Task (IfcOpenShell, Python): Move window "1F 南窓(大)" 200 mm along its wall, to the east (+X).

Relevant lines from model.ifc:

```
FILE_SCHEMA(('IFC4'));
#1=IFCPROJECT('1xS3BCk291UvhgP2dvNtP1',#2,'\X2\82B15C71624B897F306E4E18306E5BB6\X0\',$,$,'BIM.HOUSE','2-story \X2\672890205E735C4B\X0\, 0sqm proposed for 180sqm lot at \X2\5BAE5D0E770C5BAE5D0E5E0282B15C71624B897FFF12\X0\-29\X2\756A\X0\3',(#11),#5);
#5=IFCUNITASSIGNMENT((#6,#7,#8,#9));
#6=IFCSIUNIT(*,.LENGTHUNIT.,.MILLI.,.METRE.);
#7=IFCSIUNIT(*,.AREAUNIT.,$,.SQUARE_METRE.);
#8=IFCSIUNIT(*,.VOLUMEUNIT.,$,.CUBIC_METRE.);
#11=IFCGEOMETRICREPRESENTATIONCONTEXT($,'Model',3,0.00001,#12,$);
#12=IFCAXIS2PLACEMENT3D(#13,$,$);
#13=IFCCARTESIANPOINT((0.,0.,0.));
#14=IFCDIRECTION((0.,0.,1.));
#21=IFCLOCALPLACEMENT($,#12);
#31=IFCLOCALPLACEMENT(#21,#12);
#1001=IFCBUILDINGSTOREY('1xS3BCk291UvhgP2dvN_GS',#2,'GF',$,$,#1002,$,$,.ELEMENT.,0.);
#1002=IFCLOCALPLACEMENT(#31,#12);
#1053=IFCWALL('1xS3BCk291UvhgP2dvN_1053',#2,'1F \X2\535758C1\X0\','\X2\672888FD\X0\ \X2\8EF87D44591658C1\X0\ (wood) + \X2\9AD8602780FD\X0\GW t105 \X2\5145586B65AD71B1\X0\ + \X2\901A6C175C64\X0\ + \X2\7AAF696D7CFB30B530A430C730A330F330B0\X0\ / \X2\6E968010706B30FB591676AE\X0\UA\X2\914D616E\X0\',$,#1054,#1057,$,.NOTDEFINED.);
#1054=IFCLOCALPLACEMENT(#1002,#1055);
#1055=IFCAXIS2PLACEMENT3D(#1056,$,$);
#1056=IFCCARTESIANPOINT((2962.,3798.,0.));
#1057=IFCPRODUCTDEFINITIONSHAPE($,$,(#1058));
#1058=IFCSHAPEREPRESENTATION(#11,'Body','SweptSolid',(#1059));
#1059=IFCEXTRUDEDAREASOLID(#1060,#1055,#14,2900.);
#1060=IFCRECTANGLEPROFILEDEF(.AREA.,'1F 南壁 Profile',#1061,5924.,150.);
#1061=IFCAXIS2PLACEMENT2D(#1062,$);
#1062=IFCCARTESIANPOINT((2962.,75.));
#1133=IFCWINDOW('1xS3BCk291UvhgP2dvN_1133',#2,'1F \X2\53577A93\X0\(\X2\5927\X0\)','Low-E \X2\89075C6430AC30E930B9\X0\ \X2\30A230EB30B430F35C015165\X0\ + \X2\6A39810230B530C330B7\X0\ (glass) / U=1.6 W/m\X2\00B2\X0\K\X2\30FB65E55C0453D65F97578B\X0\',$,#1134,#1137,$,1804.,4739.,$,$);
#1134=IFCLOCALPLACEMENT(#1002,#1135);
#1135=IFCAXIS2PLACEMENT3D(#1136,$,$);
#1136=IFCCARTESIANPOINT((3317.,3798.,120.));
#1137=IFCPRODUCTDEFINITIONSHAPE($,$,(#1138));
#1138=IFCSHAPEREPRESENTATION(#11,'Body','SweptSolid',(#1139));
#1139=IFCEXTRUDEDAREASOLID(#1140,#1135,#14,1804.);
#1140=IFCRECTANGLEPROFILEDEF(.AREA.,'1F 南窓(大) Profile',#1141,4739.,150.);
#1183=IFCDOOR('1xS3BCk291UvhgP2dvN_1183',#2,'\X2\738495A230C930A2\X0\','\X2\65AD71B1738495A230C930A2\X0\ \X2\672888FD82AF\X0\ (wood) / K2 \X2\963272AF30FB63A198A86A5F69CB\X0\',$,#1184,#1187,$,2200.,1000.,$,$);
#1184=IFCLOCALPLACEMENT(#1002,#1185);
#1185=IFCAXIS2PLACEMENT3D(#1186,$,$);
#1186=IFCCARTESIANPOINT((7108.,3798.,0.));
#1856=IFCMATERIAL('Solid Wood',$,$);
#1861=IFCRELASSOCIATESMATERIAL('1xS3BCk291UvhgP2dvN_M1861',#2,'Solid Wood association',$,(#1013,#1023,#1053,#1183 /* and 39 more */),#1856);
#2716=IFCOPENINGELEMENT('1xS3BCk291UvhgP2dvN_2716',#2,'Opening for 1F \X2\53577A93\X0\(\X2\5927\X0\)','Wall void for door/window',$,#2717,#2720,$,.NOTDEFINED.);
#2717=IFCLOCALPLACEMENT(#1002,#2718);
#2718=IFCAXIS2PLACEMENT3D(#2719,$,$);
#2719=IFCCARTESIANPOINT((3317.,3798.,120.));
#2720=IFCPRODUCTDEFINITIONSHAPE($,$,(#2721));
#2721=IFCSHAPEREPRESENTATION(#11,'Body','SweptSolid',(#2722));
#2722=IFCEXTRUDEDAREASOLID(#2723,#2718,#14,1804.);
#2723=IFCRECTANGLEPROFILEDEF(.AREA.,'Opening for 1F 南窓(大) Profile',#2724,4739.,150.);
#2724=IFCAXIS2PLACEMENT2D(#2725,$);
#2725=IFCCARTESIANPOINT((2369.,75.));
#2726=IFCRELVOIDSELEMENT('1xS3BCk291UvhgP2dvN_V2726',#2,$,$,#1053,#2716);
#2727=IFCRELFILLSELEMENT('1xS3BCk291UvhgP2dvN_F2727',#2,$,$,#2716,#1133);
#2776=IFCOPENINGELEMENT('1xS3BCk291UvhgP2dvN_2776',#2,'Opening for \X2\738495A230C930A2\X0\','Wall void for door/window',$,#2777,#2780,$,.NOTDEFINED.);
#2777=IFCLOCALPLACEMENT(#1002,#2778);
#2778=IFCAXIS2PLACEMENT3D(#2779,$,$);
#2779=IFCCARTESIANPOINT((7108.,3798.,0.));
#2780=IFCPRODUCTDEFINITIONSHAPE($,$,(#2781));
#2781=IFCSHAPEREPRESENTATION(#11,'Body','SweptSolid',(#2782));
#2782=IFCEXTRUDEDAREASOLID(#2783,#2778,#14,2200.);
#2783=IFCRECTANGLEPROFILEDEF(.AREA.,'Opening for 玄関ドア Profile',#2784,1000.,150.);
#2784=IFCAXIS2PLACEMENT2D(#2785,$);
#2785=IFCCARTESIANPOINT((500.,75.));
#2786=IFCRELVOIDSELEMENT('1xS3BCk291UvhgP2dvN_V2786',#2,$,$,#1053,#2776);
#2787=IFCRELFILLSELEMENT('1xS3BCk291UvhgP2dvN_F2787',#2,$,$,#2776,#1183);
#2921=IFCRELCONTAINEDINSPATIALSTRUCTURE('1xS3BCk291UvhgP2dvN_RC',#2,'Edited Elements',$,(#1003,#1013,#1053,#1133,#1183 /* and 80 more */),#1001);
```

```python
import ifcopenshell
import ifcopenshell.api.geometry
import ifcopenshell.util.placement
import ifcopenshell.util.unit

model = ifcopenshell.open("model.ifc")
unit_scale = ifcopenshell.util.unit.calculate_unit_scale(model)

window = model.by_guid("1xS3BCk291UvhgP2dvN_1133")
opening = window.FillsVoids[0].RelatingOpeningElement
wall = opening.VoidsElements[0].RelatingBuildingElement

wall_matrix = ifcopenshell.util.placement.get_local_placement(wall.ObjectPlacement)
shift = wall_matrix[:3, 0] * 0.2 / unit_scale
before = ifcopenshell.util.placement.get_local_placement(window.ObjectPlacement)[:3, 3].copy()

# The window is not placed relative to its opening, so move both.
for product in (opening, window):
    matrix = ifcopenshell.util.placement.get_local_placement(product.ObjectPlacement)
    matrix[:3, 3] += shift
    ifcopenshell.api.geometry.edit_object_placement(model, product=product, matrix=matrix, is_si=False)

after = ifcopenshell.util.placement.get_local_placement(window.ObjectPlacement)[:3, 3]
print("window moved by", (after - before).round(3) + 0.0)

model.write("model_v2.ifc")
```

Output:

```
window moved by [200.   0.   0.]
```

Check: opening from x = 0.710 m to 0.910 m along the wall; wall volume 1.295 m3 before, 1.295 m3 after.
